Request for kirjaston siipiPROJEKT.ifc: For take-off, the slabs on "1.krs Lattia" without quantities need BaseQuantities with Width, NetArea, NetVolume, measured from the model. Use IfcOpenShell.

First a look at what the model holds.

```python
import ifcopenshell
import ifcopenshell.util.element
import ifcopenshell.util.unit

model = ifcopenshell.open("kirjaston siipiPROJEKT.ifc")
print(model.schema)
for unit_type in ("LENGTHUNIT", "AREAUNIT", "VOLUMEUNIT"):
    print(unit_type, ifcopenshell.util.unit.calculate_unit_scale(model, unit_type))
storey = next(s for s in model.by_type("IfcBuildingStorey") if s.Name == "1.krs Lattia")
slabs = [e for e in ifcopenshell.util.element.get_decomposition(storey) if e.is_a("IfcSlab")]
for e in sorted(slabs, key=lambda e: e.id()):
    print(e.id(), e.is_a(), e.Name, list(ifcopenshell.util.element.get_psets(e, qtos_only=True)), sep=" | ")
```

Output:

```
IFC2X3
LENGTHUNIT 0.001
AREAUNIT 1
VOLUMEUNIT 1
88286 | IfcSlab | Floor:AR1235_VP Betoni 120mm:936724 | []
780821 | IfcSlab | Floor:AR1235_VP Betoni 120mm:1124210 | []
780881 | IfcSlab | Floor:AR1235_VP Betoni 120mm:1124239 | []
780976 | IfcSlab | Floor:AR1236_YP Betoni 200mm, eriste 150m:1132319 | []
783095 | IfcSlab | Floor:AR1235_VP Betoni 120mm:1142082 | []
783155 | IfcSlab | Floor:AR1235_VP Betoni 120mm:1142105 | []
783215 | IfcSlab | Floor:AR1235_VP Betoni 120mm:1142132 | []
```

```python
import ifcopenshell
import ifcopenshell.api.pset
import ifcopenshell.geom
import ifcopenshell.util.element
import ifcopenshell.util.shape
import ifcopenshell.util.unit

model = ifcopenshell.open("kirjaston siipiPROJEKT.ifc")
unit_scale = ifcopenshell.util.unit.calculate_unit_scale(model)
area_scale = ifcopenshell.util.unit.calculate_unit_scale(model, "AREAUNIT")
volume_scale = ifcopenshell.util.unit.calculate_unit_scale(model, "VOLUMEUNIT")
settings = ifcopenshell.geom.settings()

storey = next(s for s in model.by_type("IfcBuildingStorey") if s.Name == "1.krs Lattia")
slabs = [e for e in ifcopenshell.util.element.get_decomposition(storey) if e.is_a("IfcSlab")]

for e in sorted(slabs, key=lambda e: e.id()):
    if ifcopenshell.util.element.get_psets(e, qtos_only=True, should_inherit=False):
        continue
    # Geometry comes back in metres, in the element's own axes.
    shape = ifcopenshell.geom.create_shape(settings, e)
    values = {
        "Width": ifcopenshell.util.shape.get_z(shape.geometry) / unit_scale,
        "NetArea": ifcopenshell.util.shape.get_footprint_area(shape.geometry) / area_scale,
        "NetVolume": ifcopenshell.util.shape.get_volume(shape.geometry) / volume_scale,
    }
    qto = ifcopenshell.api.pset.add_qto(model, product=e, name="BaseQuantities")
    ifcopenshell.api.pset.edit_qto(model, qto=qto, properties=values)
    print(e.id(), {k: round(v, 3) for k, v in values.items()})

model.write("kirjaston siipiPROJEKT_updated.ifc")
```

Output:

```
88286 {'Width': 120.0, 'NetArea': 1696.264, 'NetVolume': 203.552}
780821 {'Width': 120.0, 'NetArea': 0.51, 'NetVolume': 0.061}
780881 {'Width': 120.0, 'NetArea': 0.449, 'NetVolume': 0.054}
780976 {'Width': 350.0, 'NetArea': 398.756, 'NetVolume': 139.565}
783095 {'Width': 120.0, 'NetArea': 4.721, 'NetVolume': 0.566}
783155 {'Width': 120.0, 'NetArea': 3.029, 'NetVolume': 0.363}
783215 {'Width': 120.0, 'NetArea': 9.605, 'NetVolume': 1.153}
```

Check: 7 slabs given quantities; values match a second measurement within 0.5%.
